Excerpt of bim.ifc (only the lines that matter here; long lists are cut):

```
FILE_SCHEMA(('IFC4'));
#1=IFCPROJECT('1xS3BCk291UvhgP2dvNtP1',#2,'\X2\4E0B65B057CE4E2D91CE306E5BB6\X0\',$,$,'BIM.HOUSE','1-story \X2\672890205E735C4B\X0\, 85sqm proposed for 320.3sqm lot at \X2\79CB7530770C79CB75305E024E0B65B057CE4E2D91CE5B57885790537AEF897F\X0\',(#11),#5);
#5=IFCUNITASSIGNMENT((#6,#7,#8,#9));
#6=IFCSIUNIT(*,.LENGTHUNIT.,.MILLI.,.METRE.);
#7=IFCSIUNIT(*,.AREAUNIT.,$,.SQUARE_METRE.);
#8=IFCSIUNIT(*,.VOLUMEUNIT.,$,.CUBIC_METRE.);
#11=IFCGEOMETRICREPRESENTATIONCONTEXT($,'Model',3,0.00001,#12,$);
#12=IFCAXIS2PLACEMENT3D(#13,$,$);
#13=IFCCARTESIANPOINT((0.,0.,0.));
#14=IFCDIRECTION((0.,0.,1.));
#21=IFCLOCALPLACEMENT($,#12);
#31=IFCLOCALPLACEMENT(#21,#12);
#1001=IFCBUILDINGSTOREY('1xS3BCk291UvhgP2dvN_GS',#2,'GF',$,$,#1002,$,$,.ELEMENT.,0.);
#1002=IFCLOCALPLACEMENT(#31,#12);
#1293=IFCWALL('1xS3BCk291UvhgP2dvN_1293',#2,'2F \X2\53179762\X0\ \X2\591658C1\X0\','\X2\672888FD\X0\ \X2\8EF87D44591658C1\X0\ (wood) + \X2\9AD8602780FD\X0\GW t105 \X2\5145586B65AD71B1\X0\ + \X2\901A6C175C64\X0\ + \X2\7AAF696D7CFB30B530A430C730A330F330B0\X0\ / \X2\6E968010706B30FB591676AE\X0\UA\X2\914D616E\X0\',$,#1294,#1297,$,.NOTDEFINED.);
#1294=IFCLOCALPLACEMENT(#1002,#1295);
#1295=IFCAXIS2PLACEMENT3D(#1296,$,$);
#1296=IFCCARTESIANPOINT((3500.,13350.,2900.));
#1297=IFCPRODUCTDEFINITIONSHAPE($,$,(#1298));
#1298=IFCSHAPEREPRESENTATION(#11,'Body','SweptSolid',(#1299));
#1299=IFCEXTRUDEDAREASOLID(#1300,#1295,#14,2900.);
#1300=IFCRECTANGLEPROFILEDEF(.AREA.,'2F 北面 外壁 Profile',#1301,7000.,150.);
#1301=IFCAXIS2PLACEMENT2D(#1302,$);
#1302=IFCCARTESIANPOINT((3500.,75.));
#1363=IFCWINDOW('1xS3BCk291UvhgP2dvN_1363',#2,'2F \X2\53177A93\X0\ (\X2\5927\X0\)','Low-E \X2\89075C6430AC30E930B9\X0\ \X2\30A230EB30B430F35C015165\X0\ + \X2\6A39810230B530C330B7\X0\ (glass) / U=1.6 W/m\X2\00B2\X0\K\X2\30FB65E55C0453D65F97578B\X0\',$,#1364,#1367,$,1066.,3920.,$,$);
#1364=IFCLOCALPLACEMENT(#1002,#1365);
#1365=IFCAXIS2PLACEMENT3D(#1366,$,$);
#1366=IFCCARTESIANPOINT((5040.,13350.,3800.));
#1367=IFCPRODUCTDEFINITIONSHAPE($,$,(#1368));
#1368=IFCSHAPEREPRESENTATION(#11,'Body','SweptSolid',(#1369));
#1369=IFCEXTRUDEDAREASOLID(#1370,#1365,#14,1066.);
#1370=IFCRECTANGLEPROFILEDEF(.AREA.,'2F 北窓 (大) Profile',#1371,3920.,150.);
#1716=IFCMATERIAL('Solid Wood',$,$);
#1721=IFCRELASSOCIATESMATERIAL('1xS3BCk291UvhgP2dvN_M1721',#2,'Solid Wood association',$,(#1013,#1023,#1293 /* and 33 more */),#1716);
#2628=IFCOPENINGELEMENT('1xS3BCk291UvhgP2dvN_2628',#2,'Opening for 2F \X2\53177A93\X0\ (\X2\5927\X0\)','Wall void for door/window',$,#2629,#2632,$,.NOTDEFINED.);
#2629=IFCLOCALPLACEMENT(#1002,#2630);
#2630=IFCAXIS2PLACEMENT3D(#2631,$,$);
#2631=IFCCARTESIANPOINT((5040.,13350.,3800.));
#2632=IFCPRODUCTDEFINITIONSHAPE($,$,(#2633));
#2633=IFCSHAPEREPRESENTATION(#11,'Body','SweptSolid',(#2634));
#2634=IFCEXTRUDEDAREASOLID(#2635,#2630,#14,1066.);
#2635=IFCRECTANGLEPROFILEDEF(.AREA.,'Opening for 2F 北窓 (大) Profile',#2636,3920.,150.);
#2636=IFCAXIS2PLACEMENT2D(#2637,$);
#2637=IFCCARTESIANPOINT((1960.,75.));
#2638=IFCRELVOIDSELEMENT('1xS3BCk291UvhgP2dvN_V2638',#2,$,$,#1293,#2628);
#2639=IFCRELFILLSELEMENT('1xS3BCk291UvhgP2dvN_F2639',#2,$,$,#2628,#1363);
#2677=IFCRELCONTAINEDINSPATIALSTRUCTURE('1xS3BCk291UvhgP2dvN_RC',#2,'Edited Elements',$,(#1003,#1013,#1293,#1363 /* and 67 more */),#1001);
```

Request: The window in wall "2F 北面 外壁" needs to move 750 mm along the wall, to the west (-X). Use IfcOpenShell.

```python
import ifcopenshell
import ifcopenshell.api.geometry
import ifcopenshell.util.placement
import ifcopenshell.util.unit

model = ifcopenshell.open("bim.ifc")
unit_scale = ifcopenshell.util.unit.calculate_unit_scale(model)

window = model.by_id(1363)
opening = window.FillsVoids[0].RelatingOpeningElement
wall = opening.VoidsElements[0].RelatingBuildingElement

wall_matrix = ifcopenshell.util.placement.get_local_placement(wall.ObjectPlacement)
shift = wall_matrix[:3, 0] * -0.75 / unit_scale
before = ifcopenshell.util.placement.get_local_placement(window.ObjectPlacement)[:3, 3].copy()

# The window is not placed relative to its opening, so move both.
for product in (opening, window):
    matrix = ifcopenshell.util.placement.get_local_placement(product.ObjectPlacement)
    matrix[:3, 3] += shift
    ifcopenshell.api.geometry.edit_object_placement(model, product=product, matrix=matrix, is_si=False)

after = ifcopenshell.util.placement.get_local_placement(window.ObjectPlacement)[:3, 3]
print("window moved by", (after - before).round(3) + 0.0)

model.write("bim-out.ifc")
```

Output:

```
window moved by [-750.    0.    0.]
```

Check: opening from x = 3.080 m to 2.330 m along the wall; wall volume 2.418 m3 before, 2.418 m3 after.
